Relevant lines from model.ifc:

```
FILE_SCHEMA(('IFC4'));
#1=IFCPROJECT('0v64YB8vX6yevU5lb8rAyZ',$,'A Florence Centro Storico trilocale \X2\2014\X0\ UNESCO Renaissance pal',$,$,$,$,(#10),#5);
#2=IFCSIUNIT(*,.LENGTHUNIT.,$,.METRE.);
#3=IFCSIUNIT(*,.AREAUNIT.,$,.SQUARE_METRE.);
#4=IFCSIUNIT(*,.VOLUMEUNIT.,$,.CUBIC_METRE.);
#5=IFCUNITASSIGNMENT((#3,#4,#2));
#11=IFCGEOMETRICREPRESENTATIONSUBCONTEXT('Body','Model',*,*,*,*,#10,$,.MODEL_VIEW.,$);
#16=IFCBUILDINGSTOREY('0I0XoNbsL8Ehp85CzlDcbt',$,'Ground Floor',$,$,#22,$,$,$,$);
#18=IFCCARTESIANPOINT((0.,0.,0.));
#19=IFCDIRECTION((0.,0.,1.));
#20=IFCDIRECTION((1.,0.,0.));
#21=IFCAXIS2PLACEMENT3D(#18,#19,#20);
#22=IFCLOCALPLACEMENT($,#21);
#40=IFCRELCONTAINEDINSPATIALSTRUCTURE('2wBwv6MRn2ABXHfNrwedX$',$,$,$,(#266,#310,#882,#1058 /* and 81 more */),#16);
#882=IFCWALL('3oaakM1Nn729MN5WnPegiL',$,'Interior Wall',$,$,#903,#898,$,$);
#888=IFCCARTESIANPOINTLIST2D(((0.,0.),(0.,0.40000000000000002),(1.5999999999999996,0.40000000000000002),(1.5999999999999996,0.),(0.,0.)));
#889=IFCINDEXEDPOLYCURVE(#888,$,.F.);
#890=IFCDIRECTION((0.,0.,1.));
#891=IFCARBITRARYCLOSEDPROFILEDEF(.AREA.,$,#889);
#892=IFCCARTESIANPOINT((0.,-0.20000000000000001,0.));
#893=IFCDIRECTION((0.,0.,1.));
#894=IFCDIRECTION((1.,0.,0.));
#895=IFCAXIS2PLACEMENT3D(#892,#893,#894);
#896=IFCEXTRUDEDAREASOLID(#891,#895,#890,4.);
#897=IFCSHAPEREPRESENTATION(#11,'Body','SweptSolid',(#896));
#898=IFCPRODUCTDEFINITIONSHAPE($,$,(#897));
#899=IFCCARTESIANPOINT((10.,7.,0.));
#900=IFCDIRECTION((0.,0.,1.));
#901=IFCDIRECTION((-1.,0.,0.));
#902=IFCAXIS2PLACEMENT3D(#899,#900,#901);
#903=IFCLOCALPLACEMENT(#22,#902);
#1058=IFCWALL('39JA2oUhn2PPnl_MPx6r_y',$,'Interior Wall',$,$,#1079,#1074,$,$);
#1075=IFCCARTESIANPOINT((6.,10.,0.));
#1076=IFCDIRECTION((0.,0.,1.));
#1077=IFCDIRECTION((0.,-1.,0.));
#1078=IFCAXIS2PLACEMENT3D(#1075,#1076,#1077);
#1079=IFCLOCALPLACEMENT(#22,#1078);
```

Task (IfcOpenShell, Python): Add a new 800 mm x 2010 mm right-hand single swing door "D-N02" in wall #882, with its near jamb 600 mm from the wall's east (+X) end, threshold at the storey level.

```python
import numpy as np
import ifcopenshell
import ifcopenshell.api.feature
import ifcopenshell.api.geometry
import ifcopenshell.api.root
import ifcopenshell.api.spatial
import ifcopenshell.geom
import ifcopenshell.util.element
import ifcopenshell.util.placement
import ifcopenshell.util.representation
import ifcopenshell.util.shape
import ifcopenshell.util.unit

model = ifcopenshell.open("model.ifc")
unit_scale = ifcopenshell.util.unit.calculate_unit_scale(model)
settings = ifcopenshell.geom.settings()


def volume(element):
    """Net volume in cubic metres, openings subtracted."""
    shape = ifcopenshell.geom.create_shape(settings, element)
    return ifcopenshell.util.shape.get_volume(shape.geometry)


wall = model.by_guid("3oaakM1Nn729MN5WnPegiL")
storey = ifcopenshell.util.element.get_container(wall, ifc_class="IfcBuildingStorey")
context = ifcopenshell.util.representation.get_context(model, "Model", "Body", "MODEL_VIEW")
before = volume(wall)

width, height, from_end, sill = 0.8, 2.01, 0.6, 0.0  # metres

# The wall runs along its own X axis, and the end named is its -X end.
wall_shape = ifcopenshell.geom.create_shape(settings, wall)
x, y, z = ifcopenshell.util.shape.get_vertices(wall_shape.geometry).T
start = x.min() + from_end
face, thickness = float(y.min()), float(y.max() - y.min())
wall_matrix = ifcopenshell.util.placement.get_local_placement(wall.ObjectPlacement)
level = ifcopenshell.util.placement.get_local_placement(storey.ObjectPlacement)[2, 3]


def in_wall(x, y):
    """Placement at x, y metres in the wall's axes, at sill height."""
    matrix = wall_matrix.copy()
    matrix[:, 3] = wall_matrix @ np.array([x / unit_scale, y / unit_scale, 0.0, 1.0])
    matrix[2, 3] = level + sill / unit_scale
    return matrix


# Opening: a box that overshoots both wall faces by 50 mm.
opening = ifcopenshell.api.root.create_entity(model, ifc_class="IfcOpeningElement", predefined_type="OPENING")
box = ifcopenshell.api.geometry.add_wall_representation(
    model, context=context, length=width, height=height, thickness=thickness + 0.1
)
ifcopenshell.api.geometry.assign_representation(model, product=opening, representation=box)
ifcopenshell.api.geometry.edit_object_placement(model, product=opening, matrix=in_wall(start, face - 0.05), is_si=False)
ifcopenshell.api.feature.add_feature(model, feature=opening, element=wall)

door = ifcopenshell.api.root.create_entity(model, ifc_class="IfcDoor", name="D-N02", predefined_type="DOOR")
door.OverallWidth, door.OverallHeight = width / unit_scale, height / unit_scale
door.OperationType = "SINGLE_SWING_RIGHT"
body = ifcopenshell.api.geometry.add_door_representation(
    model,
    context=context,
    overall_width=door.OverallWidth,
    overall_height=door.OverallHeight,
    operation_type="SINGLE_SWING_RIGHT",
    lining_properties={"LiningDepth": thickness / unit_scale, "ThresholdDepth": thickness / unit_scale},
)
ifcopenshell.api.geometry.assign_representation(model, product=door, representation=body)
ifcopenshell.api.spatial.assign_container(model, products=[door], relating_structure=storey)
ifcopenshell.api.feature.add_filling(model, opening=opening, element=door)

# The lining spans the wall, so the door starts at the wall face.
ifcopenshell.api.geometry.edit_object_placement(model, product=door, matrix=in_wall(start, face), is_si=False)

after = volume(wall)

print(f"wall volume {before:.3f} -> {after:.3f} m3")

model.write("model_edited.ifc")
```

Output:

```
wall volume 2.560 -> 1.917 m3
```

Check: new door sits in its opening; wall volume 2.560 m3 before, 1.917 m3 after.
